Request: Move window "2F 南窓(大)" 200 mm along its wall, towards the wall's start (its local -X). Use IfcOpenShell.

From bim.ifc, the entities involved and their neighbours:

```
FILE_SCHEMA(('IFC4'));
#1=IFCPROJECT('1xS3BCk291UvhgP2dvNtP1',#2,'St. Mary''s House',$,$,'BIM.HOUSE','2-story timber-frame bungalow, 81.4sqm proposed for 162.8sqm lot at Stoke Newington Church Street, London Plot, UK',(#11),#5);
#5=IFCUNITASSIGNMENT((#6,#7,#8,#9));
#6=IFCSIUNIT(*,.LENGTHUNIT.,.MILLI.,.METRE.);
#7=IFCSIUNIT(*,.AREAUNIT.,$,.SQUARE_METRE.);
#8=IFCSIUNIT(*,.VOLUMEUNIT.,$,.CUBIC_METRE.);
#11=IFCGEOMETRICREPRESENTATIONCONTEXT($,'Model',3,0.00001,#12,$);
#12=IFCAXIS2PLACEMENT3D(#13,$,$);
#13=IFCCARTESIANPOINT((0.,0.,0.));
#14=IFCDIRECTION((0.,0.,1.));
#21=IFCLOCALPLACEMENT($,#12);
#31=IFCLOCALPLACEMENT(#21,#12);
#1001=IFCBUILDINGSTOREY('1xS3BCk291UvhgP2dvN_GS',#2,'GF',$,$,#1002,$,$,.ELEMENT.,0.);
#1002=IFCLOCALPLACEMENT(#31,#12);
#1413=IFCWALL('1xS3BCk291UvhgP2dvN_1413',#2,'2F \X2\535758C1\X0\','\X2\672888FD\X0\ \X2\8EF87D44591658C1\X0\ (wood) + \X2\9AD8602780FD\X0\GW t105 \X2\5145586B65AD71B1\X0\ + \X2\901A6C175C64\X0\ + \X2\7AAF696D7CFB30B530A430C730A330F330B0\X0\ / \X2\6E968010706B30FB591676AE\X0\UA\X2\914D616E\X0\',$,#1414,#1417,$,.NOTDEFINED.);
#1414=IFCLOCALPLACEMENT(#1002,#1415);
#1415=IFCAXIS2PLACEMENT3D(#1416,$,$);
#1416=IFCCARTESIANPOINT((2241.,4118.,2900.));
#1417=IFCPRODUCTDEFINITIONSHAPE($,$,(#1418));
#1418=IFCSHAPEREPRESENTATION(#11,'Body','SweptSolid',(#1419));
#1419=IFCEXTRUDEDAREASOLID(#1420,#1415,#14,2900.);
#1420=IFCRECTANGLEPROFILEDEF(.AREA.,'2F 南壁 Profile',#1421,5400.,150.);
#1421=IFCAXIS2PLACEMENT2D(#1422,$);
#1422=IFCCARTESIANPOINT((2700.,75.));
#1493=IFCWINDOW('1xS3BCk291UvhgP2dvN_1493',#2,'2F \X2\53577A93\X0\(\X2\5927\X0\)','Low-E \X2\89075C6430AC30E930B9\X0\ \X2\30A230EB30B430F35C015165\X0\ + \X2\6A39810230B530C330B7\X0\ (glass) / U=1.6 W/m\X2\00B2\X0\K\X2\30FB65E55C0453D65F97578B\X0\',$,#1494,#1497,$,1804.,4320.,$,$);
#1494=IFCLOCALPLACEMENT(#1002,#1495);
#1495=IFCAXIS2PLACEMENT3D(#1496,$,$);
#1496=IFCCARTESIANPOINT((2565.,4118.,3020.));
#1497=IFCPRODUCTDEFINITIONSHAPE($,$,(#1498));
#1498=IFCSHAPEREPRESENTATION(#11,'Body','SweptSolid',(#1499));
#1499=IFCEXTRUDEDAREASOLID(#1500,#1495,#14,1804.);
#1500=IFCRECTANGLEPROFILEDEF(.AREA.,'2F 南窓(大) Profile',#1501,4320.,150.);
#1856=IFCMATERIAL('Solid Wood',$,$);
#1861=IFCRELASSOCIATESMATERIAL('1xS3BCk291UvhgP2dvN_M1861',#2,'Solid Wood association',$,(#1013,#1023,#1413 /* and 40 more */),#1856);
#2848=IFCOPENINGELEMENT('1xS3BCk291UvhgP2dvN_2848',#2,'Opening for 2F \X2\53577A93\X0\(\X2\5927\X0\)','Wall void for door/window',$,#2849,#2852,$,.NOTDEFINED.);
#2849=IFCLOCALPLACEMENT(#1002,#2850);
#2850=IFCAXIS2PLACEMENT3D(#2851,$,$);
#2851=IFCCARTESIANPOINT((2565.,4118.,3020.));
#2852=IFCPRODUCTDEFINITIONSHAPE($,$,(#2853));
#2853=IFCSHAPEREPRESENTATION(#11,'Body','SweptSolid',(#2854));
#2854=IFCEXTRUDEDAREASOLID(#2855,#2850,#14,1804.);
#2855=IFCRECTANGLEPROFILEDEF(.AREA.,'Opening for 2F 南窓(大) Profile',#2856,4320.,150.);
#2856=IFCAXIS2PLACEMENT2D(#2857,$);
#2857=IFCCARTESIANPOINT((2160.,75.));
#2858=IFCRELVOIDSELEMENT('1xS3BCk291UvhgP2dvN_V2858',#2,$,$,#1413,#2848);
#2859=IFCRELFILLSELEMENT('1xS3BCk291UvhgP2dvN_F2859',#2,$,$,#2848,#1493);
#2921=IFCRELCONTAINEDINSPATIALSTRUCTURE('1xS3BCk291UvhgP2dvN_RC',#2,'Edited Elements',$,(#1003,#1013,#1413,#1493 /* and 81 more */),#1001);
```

```python
import ifcopenshell
import ifcopenshell.api.geometry
import ifcopenshell.util.placement

model = ifcopenshell.open("bim.ifc")

window = model.by_guid("1xS3BCk291UvhgP2dvN_1493")
opening = window.FillsVoids[0].RelatingOpeningElement
wall = opening.VoidsElements[0].RelatingBuildingElement

wall_matrix = ifcopenshell.util.placement.get_local_placement(wall.ObjectPlacement)
shift = wall_matrix[:3, 0] * -200.0
before = ifcopenshell.util.placement.get_local_placement(window.ObjectPlacement)[:3, 3].copy()

# The window is not placed relative to its opening, so move both.
for product in (opening, window):
    matrix = ifcopenshell.util.placement.get_local_placement(product.ObjectPlacement)
    matrix[:3, 3] += shift
    ifcopenshell.api.geometry.edit_object_placement(model, product=product, matrix=matrix, is_si=False)

after = ifcopenshell.util.placement.get_local_placement(window.ObjectPlacement)[:3, 3]
print("window moved by", (after - before).round(3) + 0.0)

model.write("bim_edited.ifc")
```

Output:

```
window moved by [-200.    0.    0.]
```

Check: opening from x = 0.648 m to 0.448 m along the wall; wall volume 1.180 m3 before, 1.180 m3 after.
